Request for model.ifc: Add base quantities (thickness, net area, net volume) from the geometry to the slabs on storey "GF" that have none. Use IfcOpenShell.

First a look at what the model holds.

```python
import ifcopenshell
import ifcopenshell.util.element
import ifcopenshell.util.unit

model = ifcopenshell.open("model.ifc")
print(model.schema)
for unit_type in ("LENGTHUNIT", "AREAUNIT", "VOLUMEUNIT"):
    print(unit_type, ifcopenshell.util.unit.calculate_unit_scale(model, unit_type))
storey = next(s for s in model.by_type("IfcBuildingStorey") if s.Name == "GF")
slabs = [e for e in ifcopenshell.util.element.get_decomposition(storey) if e.is_a("IfcSlab")]
for e in sorted(slabs, key=lambda e: e.id()):
    print(e.id(), e.is_a(), e.Name, list(ifcopenshell.util.element.get_psets(e, qtos_only=True)), sep=" | ")
```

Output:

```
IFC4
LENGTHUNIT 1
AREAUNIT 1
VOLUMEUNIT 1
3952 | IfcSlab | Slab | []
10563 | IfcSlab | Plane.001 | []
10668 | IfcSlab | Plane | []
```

```python
import ifcopenshell
import ifcopenshell.api.pset
import ifcopenshell.geom
import ifcopenshell.util.element
import ifcopenshell.util.shape
import ifcopenshell.util.unit

model = ifcopenshell.open("model.ifc")
unit_scale = ifcopenshell.util.unit.calculate_unit_scale(model)
area_scale = ifcopenshell.util.unit.calculate_unit_scale(model, "AREAUNIT")
volume_scale = ifcopenshell.util.unit.calculate_unit_scale(model, "VOLUMEUNIT")
settings = ifcopenshell.geom.settings()

storey = next(s for s in model.by_type("IfcBuildingStorey") if s.Name == "GF")
slabs = [e for e in ifcopenshell.util.element.get_decomposition(storey) if e.is_a("IfcSlab")]

for e in sorted(slabs, key=lambda e: e.id()):
    if ifcopenshell.util.element.get_psets(e, qtos_only=True, should_inherit=False):
        continue
    # Geometry comes back in metres, in the element's own axes.
    shape = ifcopenshell.geom.create_shape(settings, e)
    values = {
        "Width": ifcopenshell.util.shape.get_z(shape.geometry) / unit_scale,
        "NetArea": ifcopenshell.util.shape.get_footprint_area(shape.geometry) / area_scale,
        "NetVolume": ifcopenshell.util.shape.get_volume(shape.geometry) / volume_scale,
    }
    qto = ifcopenshell.api.pset.add_qto(model, product=e, name="Qto_SlabBaseQuantities")
    ifcopenshell.api.pset.edit_qto(model, qto=qto, properties=values)
    print(e.id(), {k: round(v, 3) for k, v in values.items()})

model.write("model_edited.ifc")
```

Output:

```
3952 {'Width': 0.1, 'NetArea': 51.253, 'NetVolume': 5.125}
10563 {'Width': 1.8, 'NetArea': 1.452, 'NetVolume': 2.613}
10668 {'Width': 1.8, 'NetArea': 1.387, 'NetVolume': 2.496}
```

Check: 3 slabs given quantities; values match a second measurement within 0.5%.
